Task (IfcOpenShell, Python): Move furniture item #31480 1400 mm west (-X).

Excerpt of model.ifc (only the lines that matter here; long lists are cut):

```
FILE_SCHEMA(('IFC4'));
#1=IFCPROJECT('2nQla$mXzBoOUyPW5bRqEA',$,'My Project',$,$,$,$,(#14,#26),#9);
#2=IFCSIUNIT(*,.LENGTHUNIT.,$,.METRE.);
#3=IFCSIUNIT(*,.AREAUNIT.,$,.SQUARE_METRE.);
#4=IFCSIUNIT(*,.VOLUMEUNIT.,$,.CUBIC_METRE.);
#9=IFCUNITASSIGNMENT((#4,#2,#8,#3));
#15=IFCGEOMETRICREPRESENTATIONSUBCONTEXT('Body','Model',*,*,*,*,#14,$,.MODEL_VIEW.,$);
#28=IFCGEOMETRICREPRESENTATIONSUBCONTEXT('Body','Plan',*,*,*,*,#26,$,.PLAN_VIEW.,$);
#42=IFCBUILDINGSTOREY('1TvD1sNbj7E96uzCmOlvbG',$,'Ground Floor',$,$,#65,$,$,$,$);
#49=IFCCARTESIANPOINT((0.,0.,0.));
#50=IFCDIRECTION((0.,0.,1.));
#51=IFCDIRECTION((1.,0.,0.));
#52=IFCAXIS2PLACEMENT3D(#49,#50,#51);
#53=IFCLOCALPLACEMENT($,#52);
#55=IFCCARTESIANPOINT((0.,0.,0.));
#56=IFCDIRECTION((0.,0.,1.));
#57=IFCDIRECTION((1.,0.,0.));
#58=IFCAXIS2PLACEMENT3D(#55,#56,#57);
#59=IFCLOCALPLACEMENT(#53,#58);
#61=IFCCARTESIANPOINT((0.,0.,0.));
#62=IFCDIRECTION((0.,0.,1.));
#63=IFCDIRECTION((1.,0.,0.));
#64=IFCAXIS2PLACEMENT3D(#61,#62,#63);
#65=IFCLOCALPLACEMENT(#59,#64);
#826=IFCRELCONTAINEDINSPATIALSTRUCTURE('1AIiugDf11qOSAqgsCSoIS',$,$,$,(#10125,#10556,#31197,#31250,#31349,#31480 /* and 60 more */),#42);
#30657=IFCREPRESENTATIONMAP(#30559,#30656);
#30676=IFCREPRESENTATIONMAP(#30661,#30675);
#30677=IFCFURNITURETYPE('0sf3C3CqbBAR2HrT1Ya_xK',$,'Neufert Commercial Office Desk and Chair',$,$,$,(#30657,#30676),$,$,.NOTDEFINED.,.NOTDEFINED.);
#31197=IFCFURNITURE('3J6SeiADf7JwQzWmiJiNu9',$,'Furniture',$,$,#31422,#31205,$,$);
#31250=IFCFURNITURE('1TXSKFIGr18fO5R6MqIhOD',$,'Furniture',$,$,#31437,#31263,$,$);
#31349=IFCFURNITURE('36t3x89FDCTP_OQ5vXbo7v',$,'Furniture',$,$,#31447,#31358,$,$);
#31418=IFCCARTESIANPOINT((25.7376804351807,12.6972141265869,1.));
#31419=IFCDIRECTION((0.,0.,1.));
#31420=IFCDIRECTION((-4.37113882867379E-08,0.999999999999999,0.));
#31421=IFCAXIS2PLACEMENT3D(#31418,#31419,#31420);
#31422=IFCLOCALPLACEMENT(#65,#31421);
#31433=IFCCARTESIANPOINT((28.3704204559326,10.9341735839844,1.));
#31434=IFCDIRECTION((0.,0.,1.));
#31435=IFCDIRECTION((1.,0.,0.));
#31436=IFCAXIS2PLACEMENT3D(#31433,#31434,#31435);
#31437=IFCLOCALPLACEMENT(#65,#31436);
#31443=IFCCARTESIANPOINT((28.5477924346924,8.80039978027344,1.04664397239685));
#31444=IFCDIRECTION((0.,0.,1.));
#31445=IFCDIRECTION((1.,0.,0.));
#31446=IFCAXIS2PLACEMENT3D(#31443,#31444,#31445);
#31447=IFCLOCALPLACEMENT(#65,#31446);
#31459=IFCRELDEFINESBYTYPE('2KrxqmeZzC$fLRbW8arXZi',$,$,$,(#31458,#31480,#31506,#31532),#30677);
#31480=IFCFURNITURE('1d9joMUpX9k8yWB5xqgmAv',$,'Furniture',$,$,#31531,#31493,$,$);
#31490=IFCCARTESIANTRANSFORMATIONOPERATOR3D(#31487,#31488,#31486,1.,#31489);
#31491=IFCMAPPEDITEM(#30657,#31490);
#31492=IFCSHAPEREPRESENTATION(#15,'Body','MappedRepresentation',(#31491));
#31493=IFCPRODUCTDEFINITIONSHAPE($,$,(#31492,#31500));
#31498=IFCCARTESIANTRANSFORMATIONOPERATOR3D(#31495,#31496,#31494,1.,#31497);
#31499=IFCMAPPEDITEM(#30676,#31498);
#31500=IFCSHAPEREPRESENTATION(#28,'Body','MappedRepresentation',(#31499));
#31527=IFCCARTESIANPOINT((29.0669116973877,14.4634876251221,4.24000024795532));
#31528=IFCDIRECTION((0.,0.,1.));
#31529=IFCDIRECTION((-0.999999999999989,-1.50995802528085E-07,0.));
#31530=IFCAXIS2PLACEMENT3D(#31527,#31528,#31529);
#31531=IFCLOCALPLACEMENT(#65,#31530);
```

```python
import ifcopenshell
import ifcopenshell.api.geometry
import ifcopenshell.util.placement
import ifcopenshell.util.unit

model = ifcopenshell.open("model.ifc")
unit_scale = ifcopenshell.util.unit.calculate_unit_scale(model)

item = model.by_id(31480)
matrix = ifcopenshell.util.placement.get_local_placement(item.ObjectPlacement)
matrix[0, 3] -= 1.4 / unit_scale
ifcopenshell.api.geometry.edit_object_placement(model, product=item, matrix=matrix, is_si=False)

print(ifcopenshell.util.placement.get_local_placement(item.ObjectPlacement).round(3) + 0.0)

model.write("model_rev.ifc")
```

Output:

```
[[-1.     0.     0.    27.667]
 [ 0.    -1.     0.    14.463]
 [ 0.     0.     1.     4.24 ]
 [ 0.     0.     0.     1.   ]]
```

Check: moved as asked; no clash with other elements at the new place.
